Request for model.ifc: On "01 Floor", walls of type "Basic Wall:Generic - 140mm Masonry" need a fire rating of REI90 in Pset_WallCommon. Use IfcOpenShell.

First a look at what the model holds.

```python
import ifcopenshell
import ifcopenshell.util.element

model = ifcopenshell.open("model.ifc")
print(model.schema)
storey = next(s for s in model.by_type("IfcBuildingStorey") if s.Name == "01 Floor")
walls = [e for e in ifcopenshell.util.element.get_decomposition(storey) if e.is_a("IfcWall")]
seen = {}
for e in walls:
    element_type = ifcopenshell.util.element.get_type(e)
    key = (element_type.Name if element_type != e and element_type else None, ifcopenshell.util.element.get_pset(e, "Pset_WallCommon", "FireRating"))
    seen[key] = seen.get(key, 0) + 1
for (name, value), count in sorted(seen.items(), key=str):
    print(count, "x", name, "|", value)
```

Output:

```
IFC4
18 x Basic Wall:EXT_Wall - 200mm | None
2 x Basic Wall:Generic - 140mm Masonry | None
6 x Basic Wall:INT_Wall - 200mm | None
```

```python
import ifcopenshell
import ifcopenshell.api.pset
import ifcopenshell.util.element

model = ifcopenshell.open("model.ifc")

storey = next(s for s in model.by_type("IfcBuildingStorey") if s.Name == "01 Floor")
walls = [e for e in ifcopenshell.util.element.get_decomposition(storey) if e.is_a("IfcWall")]

count = 0
for e in walls:
    element_type = ifcopenshell.util.element.get_type(e)
    if element_type in (None, e) or element_type.Name != "Basic Wall:Generic - 140mm Masonry":
        continue
    # add_pset returns the element's existing set when there is one.
    pset = ifcopenshell.api.pset.add_pset(model, product=e, name="Pset_WallCommon")
    ifcopenshell.api.pset.edit_pset(model, pset=pset, properties={"FireRating": "REI90"})
    count += 1

print(count, "walls updated")

model.write("model-out.ifc")
```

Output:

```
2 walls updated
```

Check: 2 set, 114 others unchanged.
